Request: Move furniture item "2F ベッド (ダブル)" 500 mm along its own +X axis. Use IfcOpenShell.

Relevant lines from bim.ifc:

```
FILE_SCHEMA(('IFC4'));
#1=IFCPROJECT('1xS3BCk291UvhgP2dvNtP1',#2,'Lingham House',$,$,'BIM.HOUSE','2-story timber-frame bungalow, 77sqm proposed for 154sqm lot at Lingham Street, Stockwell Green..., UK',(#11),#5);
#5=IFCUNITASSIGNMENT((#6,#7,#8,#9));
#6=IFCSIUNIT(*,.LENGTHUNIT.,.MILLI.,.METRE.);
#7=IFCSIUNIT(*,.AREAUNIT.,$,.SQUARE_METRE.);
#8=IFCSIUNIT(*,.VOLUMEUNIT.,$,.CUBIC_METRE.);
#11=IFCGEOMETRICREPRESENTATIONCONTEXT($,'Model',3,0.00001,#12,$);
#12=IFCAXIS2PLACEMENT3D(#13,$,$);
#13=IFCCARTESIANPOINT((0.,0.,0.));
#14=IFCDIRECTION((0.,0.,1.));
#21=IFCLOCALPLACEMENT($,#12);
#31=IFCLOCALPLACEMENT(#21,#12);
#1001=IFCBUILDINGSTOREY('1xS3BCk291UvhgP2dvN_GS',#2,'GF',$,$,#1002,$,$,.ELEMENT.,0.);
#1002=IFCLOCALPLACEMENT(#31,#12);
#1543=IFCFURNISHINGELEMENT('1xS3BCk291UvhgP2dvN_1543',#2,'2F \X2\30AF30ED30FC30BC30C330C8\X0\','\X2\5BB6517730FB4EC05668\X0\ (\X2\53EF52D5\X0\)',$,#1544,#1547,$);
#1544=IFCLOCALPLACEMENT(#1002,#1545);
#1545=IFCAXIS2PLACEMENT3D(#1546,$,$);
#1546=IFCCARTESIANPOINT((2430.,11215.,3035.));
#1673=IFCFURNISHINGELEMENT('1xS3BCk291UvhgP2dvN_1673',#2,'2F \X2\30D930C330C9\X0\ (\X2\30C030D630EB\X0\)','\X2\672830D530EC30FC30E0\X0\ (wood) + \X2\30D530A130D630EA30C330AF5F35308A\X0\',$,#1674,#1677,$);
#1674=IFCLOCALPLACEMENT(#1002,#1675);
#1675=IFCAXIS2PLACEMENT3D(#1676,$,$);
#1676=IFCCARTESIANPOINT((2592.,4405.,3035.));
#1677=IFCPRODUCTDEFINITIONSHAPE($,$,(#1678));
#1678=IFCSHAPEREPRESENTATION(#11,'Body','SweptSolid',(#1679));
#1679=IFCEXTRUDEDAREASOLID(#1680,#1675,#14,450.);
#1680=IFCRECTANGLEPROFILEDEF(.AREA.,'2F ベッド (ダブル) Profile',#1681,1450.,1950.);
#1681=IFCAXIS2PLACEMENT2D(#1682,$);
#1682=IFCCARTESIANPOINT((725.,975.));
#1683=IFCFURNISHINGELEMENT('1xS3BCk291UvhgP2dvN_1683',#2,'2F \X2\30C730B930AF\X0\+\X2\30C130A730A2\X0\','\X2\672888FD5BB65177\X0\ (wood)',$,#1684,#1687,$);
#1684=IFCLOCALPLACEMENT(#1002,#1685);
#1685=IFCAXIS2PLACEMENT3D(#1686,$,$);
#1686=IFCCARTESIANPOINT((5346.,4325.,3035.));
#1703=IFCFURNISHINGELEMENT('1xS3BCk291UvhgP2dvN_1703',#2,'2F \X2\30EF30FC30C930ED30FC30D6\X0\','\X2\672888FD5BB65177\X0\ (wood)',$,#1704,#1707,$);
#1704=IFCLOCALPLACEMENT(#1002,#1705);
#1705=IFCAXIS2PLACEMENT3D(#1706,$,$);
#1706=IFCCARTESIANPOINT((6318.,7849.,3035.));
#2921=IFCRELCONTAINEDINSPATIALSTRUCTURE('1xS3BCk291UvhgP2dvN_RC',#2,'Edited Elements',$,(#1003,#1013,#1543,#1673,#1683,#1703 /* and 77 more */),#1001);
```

```python
import ifcopenshell
import ifcopenshell.api.geometry
import ifcopenshell.util.placement
import ifcopenshell.util.unit

model = ifcopenshell.open("bim.ifc")
unit_scale = ifcopenshell.util.unit.calculate_unit_scale(model)

item = model.by_guid("1xS3BCk291UvhgP2dvN_1673")
matrix = ifcopenshell.util.placement.get_local_placement(item.ObjectPlacement)
matrix[:3, 3] += matrix[:3, 0] * 0.5 / unit_scale
ifcopenshell.api.geometry.edit_object_placement(model, product=item, matrix=matrix, is_si=False)

print(ifcopenshell.util.placement.get_local_placement(item.ObjectPlacement).round(3) + 0.0)

model.write("bim-out.ifc")
```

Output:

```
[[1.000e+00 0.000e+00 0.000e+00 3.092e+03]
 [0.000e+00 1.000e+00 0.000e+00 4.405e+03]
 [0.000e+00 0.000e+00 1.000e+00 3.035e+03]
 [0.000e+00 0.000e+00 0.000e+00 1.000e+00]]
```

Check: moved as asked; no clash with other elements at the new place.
